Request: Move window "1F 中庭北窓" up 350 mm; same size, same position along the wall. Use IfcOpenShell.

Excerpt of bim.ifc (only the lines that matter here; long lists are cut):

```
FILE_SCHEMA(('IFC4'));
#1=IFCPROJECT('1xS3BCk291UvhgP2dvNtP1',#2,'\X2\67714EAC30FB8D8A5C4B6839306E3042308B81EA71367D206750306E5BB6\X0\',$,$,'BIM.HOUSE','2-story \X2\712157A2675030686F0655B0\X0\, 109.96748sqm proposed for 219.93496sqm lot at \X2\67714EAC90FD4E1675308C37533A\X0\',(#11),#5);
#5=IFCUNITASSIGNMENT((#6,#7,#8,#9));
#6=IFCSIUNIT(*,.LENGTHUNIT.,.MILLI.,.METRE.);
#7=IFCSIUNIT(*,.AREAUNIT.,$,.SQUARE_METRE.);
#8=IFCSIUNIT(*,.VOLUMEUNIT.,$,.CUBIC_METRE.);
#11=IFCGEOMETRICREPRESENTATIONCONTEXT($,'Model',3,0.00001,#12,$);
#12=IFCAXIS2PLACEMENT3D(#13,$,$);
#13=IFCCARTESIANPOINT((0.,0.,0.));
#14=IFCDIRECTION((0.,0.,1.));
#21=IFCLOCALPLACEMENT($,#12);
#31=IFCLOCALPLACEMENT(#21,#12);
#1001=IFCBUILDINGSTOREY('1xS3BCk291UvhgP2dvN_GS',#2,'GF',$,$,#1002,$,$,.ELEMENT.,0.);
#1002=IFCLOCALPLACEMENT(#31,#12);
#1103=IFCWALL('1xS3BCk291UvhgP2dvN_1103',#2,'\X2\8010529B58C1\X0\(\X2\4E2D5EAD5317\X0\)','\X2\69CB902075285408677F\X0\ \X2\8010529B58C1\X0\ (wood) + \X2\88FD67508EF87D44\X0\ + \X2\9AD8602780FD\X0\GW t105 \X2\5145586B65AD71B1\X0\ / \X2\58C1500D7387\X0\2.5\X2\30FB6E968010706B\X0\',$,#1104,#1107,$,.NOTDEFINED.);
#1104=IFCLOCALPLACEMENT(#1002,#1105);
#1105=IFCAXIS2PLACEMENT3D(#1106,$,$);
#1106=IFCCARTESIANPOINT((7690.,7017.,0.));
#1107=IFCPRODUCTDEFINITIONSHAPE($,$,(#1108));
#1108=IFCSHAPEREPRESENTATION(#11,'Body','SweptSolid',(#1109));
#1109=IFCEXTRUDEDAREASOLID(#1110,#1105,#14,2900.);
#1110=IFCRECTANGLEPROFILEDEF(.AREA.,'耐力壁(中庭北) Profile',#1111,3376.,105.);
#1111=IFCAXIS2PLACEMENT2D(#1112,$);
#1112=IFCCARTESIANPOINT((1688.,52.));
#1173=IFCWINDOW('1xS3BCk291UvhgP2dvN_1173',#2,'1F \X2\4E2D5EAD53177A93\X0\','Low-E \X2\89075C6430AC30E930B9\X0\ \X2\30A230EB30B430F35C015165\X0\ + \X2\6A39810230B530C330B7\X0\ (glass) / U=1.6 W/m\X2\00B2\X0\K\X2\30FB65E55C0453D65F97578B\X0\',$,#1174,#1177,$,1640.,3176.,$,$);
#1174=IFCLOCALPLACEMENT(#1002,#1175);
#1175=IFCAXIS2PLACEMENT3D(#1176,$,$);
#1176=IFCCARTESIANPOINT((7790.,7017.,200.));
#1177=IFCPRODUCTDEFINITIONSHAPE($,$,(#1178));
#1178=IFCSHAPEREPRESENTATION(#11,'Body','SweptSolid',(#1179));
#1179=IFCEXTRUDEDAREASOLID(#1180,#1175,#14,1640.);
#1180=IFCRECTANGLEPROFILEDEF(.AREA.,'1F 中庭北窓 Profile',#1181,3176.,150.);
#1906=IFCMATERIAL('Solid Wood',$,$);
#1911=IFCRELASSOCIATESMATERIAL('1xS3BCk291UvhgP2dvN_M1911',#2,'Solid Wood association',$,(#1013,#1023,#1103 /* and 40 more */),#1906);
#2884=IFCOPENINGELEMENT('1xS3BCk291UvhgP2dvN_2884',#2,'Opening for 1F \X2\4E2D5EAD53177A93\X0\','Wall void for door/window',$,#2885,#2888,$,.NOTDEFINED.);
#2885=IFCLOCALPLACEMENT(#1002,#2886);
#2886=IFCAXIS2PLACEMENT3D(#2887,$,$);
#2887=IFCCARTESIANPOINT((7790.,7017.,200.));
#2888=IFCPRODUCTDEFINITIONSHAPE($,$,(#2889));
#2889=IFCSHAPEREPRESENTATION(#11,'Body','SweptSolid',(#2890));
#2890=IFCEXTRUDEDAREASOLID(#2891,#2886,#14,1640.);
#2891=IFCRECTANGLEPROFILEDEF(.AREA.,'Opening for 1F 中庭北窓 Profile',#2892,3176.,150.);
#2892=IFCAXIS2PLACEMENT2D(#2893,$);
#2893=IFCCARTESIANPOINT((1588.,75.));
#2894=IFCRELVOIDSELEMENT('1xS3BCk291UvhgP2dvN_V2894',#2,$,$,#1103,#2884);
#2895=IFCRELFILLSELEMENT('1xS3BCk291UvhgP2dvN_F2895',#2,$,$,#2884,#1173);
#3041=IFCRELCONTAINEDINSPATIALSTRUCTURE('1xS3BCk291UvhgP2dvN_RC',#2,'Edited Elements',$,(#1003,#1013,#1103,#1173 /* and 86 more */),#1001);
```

```python
import numpy as np
import ifcopenshell
import ifcopenshell.api.geometry
import ifcopenshell.util.placement
import ifcopenshell.util.unit

model = ifcopenshell.open("bim.ifc")
unit_scale = ifcopenshell.util.unit.calculate_unit_scale(model)

window = model.by_id(1173)
opening = window.FillsVoids[0].RelatingOpeningElement
dz = 0.35 / unit_scale

shift = np.array([0.0, 0.0, dz])
# The window is not placed relative to its opening, so move both.
for product in (opening, window):
    matrix = ifcopenshell.util.placement.get_local_placement(product.ObjectPlacement)
    matrix[:3, 3] += shift
    ifcopenshell.api.geometry.edit_object_placement(model, product=product, matrix=matrix, is_si=False)

print(f"moved by {dz * unit_scale:+.3f} m")

model.write("bim_edited.ifc")
```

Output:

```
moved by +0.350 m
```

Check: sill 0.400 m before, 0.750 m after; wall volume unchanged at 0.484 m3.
